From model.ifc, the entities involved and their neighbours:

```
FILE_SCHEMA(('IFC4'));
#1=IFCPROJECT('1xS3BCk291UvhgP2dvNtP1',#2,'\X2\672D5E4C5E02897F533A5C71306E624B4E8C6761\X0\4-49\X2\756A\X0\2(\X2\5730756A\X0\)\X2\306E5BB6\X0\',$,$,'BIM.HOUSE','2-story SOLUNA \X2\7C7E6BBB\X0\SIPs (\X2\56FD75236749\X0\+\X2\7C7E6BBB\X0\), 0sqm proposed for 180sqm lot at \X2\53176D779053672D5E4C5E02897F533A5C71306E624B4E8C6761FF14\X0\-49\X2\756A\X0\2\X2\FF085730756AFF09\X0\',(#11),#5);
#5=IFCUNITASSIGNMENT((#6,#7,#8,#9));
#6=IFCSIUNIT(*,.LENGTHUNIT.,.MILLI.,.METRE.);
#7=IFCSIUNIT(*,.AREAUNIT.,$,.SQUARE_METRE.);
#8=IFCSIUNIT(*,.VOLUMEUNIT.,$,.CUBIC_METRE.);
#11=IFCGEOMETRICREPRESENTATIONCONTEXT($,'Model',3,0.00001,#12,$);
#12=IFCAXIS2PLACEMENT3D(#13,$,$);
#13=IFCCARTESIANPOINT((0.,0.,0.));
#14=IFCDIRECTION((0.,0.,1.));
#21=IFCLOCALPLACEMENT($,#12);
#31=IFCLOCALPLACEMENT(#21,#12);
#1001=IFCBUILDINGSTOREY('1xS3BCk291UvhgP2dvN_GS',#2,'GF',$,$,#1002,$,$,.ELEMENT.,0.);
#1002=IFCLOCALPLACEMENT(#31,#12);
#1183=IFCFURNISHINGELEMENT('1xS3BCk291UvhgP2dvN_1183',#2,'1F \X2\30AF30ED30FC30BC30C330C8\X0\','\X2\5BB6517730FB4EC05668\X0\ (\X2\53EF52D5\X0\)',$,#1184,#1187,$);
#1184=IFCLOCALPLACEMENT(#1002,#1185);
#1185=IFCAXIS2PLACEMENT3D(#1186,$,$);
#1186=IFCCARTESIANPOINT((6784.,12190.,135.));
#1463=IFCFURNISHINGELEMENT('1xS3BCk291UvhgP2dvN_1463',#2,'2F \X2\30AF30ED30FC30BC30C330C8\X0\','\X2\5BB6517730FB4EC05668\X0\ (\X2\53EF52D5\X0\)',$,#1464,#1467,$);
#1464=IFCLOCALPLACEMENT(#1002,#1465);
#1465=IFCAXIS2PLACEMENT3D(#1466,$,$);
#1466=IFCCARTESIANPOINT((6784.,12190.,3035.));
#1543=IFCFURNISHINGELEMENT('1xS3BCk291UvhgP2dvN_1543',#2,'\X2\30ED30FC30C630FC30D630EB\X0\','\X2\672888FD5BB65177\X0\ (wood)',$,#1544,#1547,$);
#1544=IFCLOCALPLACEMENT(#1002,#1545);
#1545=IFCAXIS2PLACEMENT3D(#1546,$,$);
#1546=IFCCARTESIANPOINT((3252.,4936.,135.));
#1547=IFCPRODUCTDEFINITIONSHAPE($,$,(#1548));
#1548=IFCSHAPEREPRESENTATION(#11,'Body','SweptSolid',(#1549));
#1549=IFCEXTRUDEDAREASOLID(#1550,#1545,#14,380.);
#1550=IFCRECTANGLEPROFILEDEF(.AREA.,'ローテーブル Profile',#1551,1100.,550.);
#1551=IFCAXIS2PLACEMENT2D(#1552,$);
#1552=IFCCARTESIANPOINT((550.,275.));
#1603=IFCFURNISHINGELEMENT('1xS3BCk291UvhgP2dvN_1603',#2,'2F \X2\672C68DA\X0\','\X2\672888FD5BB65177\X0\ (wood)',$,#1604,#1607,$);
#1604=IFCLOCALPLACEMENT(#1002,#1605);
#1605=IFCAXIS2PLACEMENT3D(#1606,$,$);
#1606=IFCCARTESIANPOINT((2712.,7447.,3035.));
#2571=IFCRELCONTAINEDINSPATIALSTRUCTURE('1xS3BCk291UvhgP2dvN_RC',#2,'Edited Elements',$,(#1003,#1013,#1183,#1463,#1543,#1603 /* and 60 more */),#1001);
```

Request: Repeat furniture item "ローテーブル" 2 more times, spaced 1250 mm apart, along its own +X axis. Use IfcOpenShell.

```python
import ifcopenshell
import ifcopenshell.api.geometry
import ifcopenshell.api.root
import ifcopenshell.util.element
import ifcopenshell.util.placement
import ifcopenshell.util.unit

model = ifcopenshell.open("model.ifc")
unit_scale = ifcopenshell.util.unit.calculate_unit_scale(model)


def reuse_history(source, copy):
    """copy_class also copies each property set's owner history, people and application; keep the originals."""
    for rel in copy.IsDefinedBy:
        if rel.is_a("IfcRelDefinesByProperties") and (history := rel.RelatingPropertyDefinition.OwnerHistory):
            rel.RelatingPropertyDefinition.OwnerHistory = source.OwnerHistory
            ifcopenshell.util.element.remove_deep2(model, history)


source = model.by_guid("1xS3BCk291UvhgP2dvN_1543")
base = ifcopenshell.util.placement.get_local_placement(source.ObjectPlacement)
step = base[:3, 0] * 1.25 / unit_scale

for i in range(1, 3):
    copy = ifcopenshell.api.root.copy_class(model, product=source)
    copy.Representation = ifcopenshell.util.element.copy_deep(
        model, source.Representation, exclude=["IfcGeometricRepresentationContext", "IfcRepresentationMap"]
    )
    reuse_history(source, copy)
    matrix = base.copy()
    matrix[:3, 3] += i * step
    print("added at", matrix[:3, 3].round(3) + 0.0)
    ifcopenshell.api.geometry.edit_object_placement(model, product=copy, matrix=matrix, is_si=False)

model.write("model_v2.ifc")
```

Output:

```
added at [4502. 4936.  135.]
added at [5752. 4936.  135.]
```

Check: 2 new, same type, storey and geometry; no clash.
